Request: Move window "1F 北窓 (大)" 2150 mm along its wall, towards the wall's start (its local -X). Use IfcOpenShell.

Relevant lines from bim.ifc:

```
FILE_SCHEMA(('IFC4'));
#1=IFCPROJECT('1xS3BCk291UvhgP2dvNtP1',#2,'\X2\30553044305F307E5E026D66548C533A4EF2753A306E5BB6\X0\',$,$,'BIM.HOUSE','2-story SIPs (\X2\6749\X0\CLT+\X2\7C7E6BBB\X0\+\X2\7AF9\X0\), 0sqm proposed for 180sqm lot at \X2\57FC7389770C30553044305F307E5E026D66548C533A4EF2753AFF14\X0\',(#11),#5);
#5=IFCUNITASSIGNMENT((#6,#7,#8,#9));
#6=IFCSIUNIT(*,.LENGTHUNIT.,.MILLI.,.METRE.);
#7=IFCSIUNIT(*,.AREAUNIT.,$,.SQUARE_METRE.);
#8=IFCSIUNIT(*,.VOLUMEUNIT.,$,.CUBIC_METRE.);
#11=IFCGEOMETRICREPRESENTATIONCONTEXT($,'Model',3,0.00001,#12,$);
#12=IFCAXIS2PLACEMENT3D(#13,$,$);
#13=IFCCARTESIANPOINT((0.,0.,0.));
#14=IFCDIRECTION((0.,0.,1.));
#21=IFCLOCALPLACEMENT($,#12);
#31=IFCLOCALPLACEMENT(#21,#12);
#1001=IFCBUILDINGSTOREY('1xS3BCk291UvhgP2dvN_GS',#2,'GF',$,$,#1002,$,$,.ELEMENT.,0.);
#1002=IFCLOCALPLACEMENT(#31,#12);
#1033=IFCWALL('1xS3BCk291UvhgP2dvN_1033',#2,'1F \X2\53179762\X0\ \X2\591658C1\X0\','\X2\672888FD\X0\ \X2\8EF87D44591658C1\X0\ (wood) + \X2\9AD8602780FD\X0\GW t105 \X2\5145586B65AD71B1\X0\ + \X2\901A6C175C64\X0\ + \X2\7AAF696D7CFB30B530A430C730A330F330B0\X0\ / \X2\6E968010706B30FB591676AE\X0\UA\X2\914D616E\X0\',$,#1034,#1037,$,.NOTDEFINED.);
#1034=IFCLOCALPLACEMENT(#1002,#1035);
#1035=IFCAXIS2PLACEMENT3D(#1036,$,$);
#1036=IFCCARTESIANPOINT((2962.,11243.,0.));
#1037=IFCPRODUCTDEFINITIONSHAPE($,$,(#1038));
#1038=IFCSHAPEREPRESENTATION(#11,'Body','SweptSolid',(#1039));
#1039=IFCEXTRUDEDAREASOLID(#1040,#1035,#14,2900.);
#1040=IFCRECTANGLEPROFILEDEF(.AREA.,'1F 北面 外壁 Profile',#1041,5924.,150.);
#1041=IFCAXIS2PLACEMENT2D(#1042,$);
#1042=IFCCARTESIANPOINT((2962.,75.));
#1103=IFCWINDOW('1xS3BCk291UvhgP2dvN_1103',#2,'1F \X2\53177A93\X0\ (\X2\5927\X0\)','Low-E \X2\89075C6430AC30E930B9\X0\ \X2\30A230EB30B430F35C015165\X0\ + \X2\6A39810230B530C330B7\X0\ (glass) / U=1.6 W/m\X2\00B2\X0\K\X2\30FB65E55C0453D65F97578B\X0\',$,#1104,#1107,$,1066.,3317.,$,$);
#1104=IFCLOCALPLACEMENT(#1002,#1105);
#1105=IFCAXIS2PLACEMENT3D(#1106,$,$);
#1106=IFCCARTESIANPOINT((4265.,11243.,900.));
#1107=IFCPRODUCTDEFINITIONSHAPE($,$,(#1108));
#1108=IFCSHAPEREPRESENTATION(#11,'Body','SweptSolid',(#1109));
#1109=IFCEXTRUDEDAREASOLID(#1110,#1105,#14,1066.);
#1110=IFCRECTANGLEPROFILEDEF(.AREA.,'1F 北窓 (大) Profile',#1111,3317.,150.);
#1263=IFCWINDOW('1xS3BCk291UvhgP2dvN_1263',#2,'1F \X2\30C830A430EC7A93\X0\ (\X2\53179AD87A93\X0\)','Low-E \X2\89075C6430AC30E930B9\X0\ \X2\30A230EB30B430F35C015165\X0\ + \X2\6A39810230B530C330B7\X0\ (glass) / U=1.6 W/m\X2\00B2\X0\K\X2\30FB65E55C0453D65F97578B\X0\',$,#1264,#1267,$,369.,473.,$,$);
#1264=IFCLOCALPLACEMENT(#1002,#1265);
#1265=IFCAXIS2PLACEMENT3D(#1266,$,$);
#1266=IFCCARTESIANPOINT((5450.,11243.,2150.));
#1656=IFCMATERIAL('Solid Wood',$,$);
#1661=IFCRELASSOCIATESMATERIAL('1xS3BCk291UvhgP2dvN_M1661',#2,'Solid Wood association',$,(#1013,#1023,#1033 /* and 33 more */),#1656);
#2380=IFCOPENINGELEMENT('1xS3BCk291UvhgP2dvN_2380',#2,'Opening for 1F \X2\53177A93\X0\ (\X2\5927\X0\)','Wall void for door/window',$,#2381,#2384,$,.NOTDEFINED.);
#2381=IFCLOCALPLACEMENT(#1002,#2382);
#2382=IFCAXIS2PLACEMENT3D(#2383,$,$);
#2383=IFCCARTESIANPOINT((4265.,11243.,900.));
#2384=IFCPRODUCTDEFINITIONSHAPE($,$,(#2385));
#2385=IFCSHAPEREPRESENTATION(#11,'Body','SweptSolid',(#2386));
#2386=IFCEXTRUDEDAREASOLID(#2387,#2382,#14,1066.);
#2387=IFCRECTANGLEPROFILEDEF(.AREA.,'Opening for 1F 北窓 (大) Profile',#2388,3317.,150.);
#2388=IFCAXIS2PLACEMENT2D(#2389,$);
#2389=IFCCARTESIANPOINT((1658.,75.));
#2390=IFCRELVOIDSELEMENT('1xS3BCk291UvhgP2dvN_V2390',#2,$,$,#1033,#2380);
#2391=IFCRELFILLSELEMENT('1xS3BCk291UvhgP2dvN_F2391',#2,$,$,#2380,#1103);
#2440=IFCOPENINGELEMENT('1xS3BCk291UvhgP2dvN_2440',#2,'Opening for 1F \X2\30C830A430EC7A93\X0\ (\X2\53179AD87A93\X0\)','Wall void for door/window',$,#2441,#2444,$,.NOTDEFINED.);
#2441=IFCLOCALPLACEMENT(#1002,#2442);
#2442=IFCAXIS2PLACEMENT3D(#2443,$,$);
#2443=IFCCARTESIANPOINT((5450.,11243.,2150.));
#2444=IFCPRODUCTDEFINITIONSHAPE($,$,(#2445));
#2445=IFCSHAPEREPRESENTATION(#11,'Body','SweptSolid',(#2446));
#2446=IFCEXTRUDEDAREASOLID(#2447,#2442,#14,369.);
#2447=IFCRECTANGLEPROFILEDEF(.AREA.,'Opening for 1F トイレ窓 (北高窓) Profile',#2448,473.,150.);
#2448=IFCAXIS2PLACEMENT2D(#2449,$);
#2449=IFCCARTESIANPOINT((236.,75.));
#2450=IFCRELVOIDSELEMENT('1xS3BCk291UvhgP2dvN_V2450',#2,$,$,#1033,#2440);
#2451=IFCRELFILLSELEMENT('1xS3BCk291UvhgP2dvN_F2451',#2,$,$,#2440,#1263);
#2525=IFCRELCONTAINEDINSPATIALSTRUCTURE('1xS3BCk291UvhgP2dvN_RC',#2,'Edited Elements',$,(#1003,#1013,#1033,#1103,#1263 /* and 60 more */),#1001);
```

```python
import ifcopenshell
import ifcopenshell.api.geometry
import ifcopenshell.util.placement

model = ifcopenshell.open("bim.ifc")

window = model.by_guid("1xS3BCk291UvhgP2dvN_1103")
opening = window.FillsVoids[0].RelatingOpeningElement
wall = opening.VoidsElements[0].RelatingBuildingElement

wall_matrix = ifcopenshell.util.placement.get_local_placement(wall.ObjectPlacement)
shift = wall_matrix[:3, 0] * -2150.0
before = ifcopenshell.util.placement.get_local_placement(window.ObjectPlacement)[:3, 3].copy()

# The window is not placed relative to its opening, so move both.
for product in (opening, window):
    matrix = ifcopenshell.util.placement.get_local_placement(product.ObjectPlacement)
    matrix[:3, 3] += shift
    ifcopenshell.api.geometry.edit_object_placement(model, product=product, matrix=matrix, is_si=False)

after = ifcopenshell.util.placement.get_local_placement(window.ObjectPlacement)[:3, 3]
print("window moved by", (after - before).round(3) + 0.0)

model.write("bim_rev.ifc")
```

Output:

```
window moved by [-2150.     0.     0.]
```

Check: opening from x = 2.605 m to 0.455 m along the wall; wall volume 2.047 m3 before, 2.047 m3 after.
